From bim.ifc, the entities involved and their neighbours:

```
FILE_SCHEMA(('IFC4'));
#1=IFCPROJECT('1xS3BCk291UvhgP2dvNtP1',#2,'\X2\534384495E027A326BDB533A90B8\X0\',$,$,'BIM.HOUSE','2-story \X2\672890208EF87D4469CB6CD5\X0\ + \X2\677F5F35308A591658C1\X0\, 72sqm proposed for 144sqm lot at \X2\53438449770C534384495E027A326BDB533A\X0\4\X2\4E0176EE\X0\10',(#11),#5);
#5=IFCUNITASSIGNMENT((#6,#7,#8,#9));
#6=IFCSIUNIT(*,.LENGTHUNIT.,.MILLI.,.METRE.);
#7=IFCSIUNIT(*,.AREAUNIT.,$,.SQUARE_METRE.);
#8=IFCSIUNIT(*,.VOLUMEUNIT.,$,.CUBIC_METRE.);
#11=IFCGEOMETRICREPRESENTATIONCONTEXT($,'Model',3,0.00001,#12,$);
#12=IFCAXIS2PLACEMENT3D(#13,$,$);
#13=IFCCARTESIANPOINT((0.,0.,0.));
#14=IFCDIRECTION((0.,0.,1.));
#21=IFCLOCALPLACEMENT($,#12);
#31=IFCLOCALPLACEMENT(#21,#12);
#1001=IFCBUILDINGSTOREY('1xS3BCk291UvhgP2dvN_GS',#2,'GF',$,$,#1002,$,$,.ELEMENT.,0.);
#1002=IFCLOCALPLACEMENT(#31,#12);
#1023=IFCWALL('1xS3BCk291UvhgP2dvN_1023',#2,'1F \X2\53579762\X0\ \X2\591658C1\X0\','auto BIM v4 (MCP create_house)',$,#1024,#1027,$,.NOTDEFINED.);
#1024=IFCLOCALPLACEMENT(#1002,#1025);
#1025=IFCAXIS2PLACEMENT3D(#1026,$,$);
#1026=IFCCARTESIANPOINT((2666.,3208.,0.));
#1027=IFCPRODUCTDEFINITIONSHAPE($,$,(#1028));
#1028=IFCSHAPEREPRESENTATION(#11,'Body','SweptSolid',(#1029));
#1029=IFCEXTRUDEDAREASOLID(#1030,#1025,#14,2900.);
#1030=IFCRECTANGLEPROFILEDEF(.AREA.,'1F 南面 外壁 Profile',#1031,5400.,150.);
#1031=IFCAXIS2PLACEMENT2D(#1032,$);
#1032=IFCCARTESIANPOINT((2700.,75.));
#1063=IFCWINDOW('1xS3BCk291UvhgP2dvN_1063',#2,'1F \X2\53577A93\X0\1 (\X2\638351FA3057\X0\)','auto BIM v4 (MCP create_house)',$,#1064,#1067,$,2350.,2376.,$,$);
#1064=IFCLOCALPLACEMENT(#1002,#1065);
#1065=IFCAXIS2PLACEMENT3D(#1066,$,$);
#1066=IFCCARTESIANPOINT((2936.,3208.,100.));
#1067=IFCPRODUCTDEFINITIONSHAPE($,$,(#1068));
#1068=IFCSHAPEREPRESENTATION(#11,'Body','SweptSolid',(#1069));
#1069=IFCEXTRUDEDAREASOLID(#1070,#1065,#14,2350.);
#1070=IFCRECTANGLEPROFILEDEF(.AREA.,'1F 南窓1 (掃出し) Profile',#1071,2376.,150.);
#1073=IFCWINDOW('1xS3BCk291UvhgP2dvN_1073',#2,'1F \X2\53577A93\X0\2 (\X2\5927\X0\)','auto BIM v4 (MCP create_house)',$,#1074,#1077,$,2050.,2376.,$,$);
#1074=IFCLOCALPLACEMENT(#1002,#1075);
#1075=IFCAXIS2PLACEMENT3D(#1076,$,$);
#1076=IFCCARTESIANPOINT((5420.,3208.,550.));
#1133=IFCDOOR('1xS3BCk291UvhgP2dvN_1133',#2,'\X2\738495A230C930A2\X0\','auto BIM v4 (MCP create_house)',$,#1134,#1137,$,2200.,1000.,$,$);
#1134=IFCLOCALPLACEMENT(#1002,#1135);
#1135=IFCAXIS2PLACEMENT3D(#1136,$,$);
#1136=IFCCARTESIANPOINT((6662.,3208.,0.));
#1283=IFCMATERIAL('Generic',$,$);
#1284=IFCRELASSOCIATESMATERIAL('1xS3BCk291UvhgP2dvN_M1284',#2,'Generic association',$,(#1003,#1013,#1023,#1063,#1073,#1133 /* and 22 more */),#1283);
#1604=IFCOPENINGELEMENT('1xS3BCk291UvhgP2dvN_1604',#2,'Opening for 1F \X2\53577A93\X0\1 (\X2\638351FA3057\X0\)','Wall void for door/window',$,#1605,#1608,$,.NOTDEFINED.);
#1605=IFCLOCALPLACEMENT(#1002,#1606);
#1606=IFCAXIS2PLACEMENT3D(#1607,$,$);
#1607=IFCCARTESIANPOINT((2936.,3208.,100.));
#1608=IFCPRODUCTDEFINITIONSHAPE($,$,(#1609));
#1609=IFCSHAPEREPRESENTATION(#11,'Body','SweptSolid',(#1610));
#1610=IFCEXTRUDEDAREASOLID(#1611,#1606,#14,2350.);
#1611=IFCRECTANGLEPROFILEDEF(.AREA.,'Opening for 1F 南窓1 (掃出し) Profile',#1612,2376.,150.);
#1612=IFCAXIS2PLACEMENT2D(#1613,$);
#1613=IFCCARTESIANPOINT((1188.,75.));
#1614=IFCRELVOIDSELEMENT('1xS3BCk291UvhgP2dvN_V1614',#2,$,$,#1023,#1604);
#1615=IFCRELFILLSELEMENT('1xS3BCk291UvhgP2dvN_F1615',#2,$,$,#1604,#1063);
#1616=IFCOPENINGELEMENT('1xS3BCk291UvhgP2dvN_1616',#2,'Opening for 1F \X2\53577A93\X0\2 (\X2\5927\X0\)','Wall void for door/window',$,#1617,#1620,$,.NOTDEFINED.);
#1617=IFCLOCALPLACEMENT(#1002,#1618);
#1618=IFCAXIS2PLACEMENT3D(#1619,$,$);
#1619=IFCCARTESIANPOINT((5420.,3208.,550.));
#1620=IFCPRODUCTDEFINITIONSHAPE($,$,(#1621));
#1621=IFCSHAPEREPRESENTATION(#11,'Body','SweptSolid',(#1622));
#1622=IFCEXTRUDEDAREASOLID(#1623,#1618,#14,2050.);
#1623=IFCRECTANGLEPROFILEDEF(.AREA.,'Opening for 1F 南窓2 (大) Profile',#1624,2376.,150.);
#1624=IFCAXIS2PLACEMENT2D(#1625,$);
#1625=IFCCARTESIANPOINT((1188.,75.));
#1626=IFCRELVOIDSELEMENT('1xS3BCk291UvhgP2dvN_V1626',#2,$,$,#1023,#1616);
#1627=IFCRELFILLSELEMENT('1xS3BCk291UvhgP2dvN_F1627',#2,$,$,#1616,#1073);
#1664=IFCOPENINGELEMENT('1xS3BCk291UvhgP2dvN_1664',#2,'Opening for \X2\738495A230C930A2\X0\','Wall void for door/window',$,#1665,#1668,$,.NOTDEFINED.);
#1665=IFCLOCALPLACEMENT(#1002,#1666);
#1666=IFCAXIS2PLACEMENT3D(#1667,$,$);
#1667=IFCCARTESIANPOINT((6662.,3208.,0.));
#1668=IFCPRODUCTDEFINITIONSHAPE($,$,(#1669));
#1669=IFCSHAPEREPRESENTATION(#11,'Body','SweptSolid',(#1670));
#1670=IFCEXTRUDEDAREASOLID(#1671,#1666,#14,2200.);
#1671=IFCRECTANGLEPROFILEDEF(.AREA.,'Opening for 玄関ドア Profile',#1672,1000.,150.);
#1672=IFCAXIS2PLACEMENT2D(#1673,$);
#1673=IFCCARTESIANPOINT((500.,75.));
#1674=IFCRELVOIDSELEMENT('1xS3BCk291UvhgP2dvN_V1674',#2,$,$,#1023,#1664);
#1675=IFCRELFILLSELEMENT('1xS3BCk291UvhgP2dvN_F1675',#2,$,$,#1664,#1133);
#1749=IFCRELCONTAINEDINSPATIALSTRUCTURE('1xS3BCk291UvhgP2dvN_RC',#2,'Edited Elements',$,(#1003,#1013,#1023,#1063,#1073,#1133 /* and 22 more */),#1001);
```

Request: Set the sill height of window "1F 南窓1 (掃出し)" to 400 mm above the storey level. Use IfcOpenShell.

```python
import numpy as np
import ifcopenshell
import ifcopenshell.api.geometry
import ifcopenshell.geom
import ifcopenshell.util.element
import ifcopenshell.util.placement
import ifcopenshell.util.shape
import ifcopenshell.util.unit

model = ifcopenshell.open("bim.ifc")
unit_scale = ifcopenshell.util.unit.calculate_unit_scale(model)

window = model.by_guid("1xS3BCk291UvhgP2dvN_1063")
opening = window.FillsVoids[0].RelatingOpeningElement
storey = ifcopenshell.util.element.get_container(window, ifc_class="IfcBuildingStorey")
level = ifcopenshell.util.placement.get_local_placement(storey.ObjectPlacement)[2, 3]

# The opening's origin need not be at the sill, so measure its lowest point.
shape = ifcopenshell.geom.create_shape(ifcopenshell.geom.settings(), opening)
bottom = ifcopenshell.util.shape.get_shape_bottom_elevation(shape, shape.geometry) / unit_scale
dz = level + 0.4 / unit_scale - bottom

shift = np.array([0.0, 0.0, dz])
# The window is not placed relative to its opening, so move both.
for product in (opening, window):
    matrix = ifcopenshell.util.placement.get_local_placement(product.ObjectPlacement)
    matrix[:3, 3] += shift
    ifcopenshell.api.geometry.edit_object_placement(model, product=product, matrix=matrix, is_si=False)

print(f"moved by {dz * unit_scale:+.3f} m")

model.write("bim_updated.ifc")
```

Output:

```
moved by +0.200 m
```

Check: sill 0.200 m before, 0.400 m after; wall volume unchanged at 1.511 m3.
